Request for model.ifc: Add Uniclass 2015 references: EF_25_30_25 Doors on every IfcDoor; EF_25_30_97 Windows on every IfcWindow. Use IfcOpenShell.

First a look at what the model holds.

```python
import ifcopenshell

model = ifcopenshell.open("model.ifc")
print(model.schema)
print("classifications:", [c.Name for c in model.by_type("IfcClassification")])
for ifc_class in ("IfcDoor", "IfcRoof", "IfcStair", "IfcWall", "IfcWindow"):
    print(ifc_class, len(model.by_type(ifc_class)))
```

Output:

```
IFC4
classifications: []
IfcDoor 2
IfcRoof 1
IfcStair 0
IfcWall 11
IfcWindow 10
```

```python
import ifcopenshell
import ifcopenshell.api.classification

model = ifcopenshell.open("model.ifc")

system = ifcopenshell.api.classification.add_classification(model, classification="Uniclass 2015")

codes = {
    "IfcDoor": ("EF_25_30_25", "Doors"),
    "IfcWindow": ("EF_25_30_97", "Windows"),
}
for ifc_class, (code, name) in codes.items():
    products = model.by_type(ifc_class)
    ifcopenshell.api.classification.add_reference(
        model, products=products, classification=system, identification=code, name=name
    )
    print(code, len(products))

model.write("model_v2.ifc")
```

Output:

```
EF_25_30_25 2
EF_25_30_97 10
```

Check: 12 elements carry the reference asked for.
